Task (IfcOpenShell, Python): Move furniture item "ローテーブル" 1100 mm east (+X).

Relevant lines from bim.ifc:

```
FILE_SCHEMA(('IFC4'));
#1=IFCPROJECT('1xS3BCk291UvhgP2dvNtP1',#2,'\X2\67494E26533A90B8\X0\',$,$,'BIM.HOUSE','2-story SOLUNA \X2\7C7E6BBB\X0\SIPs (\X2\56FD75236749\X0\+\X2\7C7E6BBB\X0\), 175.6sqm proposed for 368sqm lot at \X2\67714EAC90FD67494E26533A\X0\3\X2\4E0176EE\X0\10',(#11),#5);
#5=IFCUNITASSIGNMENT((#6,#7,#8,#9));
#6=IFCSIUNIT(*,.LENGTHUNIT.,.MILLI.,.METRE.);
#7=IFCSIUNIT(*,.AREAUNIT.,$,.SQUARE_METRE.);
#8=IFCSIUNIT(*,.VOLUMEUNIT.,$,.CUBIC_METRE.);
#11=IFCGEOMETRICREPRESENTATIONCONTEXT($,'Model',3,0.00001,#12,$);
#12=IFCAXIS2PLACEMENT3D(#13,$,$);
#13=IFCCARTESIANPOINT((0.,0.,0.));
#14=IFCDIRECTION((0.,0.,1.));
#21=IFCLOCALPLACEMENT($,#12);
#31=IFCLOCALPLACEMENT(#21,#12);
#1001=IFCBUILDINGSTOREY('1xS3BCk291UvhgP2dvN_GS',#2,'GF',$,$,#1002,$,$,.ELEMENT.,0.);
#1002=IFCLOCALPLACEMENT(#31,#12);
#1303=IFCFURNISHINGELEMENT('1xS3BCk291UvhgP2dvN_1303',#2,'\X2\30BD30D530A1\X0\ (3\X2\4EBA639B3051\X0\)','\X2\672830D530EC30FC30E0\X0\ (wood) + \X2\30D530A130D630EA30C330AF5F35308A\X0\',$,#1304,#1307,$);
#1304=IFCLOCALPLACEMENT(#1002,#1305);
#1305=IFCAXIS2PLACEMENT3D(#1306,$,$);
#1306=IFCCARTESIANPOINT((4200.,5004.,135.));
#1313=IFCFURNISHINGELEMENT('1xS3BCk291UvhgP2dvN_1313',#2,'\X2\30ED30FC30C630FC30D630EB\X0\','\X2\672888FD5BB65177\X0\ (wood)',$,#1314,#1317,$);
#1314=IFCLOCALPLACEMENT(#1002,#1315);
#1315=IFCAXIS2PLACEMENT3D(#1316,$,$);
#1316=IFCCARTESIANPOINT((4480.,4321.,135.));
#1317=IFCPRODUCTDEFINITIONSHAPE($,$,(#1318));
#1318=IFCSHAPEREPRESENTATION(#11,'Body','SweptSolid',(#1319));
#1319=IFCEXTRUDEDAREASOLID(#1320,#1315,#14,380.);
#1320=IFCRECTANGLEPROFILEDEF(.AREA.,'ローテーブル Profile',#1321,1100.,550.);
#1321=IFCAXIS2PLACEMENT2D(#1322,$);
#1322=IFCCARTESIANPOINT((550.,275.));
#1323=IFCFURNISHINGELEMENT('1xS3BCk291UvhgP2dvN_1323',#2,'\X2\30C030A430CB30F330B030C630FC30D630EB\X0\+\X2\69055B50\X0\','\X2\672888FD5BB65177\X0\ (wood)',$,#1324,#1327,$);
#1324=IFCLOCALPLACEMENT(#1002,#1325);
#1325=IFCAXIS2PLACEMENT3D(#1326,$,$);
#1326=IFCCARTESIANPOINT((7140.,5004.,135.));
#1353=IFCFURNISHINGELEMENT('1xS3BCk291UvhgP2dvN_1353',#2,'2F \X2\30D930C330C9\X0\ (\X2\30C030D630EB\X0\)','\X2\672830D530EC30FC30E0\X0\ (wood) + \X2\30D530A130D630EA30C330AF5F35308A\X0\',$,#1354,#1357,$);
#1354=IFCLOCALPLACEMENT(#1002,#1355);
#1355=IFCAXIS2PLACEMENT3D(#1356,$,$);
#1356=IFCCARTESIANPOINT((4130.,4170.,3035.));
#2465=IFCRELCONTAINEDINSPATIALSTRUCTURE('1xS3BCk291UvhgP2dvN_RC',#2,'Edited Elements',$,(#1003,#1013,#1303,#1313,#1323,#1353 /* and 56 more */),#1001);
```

```python
import ifcopenshell
import ifcopenshell.api.geometry
import ifcopenshell.util.placement
import ifcopenshell.util.unit

model = ifcopenshell.open("bim.ifc")
unit_scale = ifcopenshell.util.unit.calculate_unit_scale(model)

item = model.by_guid("1xS3BCk291UvhgP2dvN_1313")
matrix = ifcopenshell.util.placement.get_local_placement(item.ObjectPlacement)
matrix[0, 3] += 1.1 / unit_scale
ifcopenshell.api.geometry.edit_object_placement(model, product=item, matrix=matrix, is_si=False)

print(ifcopenshell.util.placement.get_local_placement(item.ObjectPlacement).round(3) + 0.0)

model.write("bim-out.ifc")
```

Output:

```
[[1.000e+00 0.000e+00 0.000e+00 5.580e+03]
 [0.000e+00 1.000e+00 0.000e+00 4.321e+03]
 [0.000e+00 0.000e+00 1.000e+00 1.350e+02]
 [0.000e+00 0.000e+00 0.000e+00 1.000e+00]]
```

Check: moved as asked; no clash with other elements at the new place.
